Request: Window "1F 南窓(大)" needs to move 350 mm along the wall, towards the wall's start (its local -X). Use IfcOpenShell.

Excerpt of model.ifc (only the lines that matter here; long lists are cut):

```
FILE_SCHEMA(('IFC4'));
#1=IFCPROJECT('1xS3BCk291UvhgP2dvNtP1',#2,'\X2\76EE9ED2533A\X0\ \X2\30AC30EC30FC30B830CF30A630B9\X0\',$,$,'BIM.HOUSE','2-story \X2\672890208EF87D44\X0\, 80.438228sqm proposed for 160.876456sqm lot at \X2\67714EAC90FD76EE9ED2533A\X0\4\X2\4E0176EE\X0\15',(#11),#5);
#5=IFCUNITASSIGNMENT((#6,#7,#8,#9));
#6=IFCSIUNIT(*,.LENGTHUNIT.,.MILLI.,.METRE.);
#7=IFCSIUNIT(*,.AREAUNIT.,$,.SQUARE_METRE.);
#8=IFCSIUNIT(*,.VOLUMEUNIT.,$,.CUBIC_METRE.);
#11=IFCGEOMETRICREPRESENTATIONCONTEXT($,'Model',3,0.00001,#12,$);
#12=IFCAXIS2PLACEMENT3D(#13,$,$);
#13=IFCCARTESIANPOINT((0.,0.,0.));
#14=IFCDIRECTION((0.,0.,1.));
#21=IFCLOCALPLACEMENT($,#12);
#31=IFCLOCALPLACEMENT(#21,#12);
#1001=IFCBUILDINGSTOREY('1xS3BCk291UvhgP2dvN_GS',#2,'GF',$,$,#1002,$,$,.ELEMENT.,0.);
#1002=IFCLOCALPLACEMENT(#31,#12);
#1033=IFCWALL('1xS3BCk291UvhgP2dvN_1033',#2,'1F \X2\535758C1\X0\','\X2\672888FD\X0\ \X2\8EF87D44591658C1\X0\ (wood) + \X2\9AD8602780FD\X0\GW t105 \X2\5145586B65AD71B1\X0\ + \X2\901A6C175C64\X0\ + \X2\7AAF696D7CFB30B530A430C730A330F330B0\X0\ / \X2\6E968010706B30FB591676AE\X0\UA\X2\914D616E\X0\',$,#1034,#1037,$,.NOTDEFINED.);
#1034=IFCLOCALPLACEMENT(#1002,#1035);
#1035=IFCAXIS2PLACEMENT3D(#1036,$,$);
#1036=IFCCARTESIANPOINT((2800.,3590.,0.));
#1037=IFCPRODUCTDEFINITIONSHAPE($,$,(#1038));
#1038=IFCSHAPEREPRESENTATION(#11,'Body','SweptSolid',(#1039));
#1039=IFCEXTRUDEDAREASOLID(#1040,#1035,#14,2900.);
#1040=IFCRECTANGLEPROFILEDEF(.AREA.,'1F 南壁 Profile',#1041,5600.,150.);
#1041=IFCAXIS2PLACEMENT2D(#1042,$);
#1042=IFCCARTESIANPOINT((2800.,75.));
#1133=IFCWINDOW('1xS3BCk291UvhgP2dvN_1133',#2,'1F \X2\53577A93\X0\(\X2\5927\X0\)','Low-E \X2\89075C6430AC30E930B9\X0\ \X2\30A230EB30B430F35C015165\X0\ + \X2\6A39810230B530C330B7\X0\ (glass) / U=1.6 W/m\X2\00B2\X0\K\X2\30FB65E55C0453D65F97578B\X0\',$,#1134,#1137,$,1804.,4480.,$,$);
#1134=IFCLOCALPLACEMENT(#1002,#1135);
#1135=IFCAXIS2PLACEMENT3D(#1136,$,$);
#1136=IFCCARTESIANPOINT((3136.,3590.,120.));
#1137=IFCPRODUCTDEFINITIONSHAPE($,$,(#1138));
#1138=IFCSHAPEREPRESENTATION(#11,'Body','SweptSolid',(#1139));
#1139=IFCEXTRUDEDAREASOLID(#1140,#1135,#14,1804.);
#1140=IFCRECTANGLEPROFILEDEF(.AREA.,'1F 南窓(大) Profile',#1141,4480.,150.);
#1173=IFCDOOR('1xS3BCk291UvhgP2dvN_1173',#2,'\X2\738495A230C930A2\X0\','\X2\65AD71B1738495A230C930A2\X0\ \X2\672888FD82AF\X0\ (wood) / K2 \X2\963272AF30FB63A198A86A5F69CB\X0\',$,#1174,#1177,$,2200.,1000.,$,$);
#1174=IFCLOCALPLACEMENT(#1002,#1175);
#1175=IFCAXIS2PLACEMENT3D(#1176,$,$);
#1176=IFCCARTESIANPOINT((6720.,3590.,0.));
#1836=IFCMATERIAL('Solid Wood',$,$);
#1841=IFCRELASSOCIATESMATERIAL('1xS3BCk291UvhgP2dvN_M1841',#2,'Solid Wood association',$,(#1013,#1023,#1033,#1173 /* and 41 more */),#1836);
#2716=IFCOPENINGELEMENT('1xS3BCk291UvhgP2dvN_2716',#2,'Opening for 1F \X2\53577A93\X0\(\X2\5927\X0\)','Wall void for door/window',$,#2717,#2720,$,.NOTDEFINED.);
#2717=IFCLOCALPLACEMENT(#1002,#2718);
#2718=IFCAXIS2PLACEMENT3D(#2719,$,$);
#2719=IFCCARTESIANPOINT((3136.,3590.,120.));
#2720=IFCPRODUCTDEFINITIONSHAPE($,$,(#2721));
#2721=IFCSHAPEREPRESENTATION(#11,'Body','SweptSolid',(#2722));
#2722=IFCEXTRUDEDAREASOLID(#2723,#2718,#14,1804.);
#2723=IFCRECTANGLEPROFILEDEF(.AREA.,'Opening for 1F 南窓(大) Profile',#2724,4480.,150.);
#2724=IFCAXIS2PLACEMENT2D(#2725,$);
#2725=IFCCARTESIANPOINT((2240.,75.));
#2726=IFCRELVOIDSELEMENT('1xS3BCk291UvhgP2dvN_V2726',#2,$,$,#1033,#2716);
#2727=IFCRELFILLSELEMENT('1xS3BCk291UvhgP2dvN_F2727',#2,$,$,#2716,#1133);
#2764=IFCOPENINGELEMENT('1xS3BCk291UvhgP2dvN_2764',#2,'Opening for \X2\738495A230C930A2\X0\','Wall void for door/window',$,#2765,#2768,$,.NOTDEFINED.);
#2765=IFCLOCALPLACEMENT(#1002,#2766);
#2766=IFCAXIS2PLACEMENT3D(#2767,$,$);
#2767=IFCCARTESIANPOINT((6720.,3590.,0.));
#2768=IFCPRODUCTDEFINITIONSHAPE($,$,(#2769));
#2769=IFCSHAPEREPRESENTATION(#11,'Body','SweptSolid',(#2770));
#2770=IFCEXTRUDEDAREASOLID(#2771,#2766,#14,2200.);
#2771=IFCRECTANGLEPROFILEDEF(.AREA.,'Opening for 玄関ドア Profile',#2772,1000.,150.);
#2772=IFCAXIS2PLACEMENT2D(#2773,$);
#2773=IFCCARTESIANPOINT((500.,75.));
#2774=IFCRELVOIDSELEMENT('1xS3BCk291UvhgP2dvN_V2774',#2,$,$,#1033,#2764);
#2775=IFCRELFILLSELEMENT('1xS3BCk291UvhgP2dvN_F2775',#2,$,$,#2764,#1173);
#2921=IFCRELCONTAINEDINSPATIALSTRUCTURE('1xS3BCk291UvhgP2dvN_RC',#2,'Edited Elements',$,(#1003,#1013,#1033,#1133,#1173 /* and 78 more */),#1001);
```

```python
import ifcopenshell
import ifcopenshell.api.geometry
import ifcopenshell.util.placement
import ifcopenshell.util.unit

model = ifcopenshell.open("model.ifc")
unit_scale = ifcopenshell.util.unit.calculate_unit_scale(model)

window = model.by_id(1133)
opening = window.FillsVoids[0].RelatingOpeningElement
wall = opening.VoidsElements[0].RelatingBuildingElement

wall_matrix = ifcopenshell.util.placement.get_local_placement(wall.ObjectPlacement)
shift = wall_matrix[:3, 0] * -0.35 / unit_scale
before = ifcopenshell.util.placement.get_local_placement(window.ObjectPlacement)[:3, 3].copy()

# The window is not placed relative to its opening, so move both.
for product in (opening, window):
    matrix = ifcopenshell.util.placement.get_local_placement(product.ObjectPlacement)
    matrix[:3, 3] += shift
    ifcopenshell.api.geometry.edit_object_placement(model, product=product, matrix=matrix, is_si=False)

after = ifcopenshell.util.placement.get_local_placement(window.ObjectPlacement)[:3, 3]
print("window moved by", (after - before).round(3) + 0.0)

model.write("model_updated.ifc")
```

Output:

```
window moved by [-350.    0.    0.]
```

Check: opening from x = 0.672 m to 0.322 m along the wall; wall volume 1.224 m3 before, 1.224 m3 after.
